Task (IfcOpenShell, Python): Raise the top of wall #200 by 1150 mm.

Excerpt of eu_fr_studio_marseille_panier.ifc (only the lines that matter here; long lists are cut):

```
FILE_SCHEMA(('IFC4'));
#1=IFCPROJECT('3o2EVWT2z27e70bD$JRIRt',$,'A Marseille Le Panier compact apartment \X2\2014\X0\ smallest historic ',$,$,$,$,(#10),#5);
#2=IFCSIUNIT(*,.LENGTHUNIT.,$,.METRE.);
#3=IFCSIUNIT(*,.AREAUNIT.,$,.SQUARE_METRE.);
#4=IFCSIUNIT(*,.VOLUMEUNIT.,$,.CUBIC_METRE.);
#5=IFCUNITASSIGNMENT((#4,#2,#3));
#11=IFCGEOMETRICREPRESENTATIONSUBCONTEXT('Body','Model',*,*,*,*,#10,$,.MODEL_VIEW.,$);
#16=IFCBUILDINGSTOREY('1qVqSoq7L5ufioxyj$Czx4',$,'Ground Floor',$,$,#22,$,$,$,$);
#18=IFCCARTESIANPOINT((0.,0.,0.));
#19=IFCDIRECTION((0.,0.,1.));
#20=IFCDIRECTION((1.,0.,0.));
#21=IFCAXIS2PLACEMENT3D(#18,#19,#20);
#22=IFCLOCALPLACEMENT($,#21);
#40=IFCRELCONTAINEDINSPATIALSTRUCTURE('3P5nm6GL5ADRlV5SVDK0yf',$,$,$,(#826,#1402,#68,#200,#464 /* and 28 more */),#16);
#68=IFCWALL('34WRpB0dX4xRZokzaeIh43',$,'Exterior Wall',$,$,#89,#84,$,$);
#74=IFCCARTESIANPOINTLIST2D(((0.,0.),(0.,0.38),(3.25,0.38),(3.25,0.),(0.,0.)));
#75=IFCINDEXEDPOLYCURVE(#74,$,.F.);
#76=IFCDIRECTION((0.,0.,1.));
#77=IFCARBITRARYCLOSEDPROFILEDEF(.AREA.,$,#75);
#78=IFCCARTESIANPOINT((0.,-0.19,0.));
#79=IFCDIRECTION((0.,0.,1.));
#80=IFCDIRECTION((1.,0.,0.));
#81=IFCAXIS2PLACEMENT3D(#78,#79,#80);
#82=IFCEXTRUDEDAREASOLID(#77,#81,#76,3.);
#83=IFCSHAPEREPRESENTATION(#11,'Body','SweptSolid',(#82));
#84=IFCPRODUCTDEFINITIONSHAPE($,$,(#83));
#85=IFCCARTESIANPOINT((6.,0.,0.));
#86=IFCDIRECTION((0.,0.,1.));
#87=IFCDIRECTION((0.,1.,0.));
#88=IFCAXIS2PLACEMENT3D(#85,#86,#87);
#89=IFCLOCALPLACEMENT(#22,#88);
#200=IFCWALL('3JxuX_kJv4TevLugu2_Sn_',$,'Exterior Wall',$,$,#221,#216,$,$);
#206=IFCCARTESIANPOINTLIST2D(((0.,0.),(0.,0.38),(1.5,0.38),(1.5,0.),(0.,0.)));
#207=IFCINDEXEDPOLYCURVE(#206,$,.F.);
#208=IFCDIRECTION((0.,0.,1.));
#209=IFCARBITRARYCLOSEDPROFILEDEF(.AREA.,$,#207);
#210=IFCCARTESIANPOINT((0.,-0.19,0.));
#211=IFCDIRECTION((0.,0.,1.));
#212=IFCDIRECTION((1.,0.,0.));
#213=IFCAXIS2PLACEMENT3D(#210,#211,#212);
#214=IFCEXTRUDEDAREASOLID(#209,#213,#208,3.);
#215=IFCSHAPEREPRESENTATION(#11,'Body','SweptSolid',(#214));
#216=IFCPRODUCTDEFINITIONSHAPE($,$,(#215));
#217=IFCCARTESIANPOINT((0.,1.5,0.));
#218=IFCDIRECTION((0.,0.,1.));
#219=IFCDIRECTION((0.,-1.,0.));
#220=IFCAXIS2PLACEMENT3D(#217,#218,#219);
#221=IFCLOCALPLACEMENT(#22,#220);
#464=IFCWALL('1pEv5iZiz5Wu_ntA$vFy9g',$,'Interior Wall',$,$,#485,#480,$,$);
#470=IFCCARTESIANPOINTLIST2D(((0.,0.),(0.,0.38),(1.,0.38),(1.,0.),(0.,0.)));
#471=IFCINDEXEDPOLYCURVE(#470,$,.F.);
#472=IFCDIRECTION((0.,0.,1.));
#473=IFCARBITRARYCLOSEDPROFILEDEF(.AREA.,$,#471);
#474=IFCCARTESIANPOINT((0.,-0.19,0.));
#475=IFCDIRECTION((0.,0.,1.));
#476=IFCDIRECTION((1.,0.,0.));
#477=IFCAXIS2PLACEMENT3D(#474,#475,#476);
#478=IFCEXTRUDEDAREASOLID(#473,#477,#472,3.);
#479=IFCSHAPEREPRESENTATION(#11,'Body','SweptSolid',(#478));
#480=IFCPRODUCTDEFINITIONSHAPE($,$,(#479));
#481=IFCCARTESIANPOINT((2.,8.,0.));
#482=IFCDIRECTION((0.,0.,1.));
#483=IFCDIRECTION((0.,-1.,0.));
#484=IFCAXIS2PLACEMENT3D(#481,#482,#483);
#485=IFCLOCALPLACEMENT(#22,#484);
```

```python
import ifcopenshell
import ifcopenshell.geom
import ifcopenshell.util.representation
import ifcopenshell.util.shape

model = ifcopenshell.open("eu_fr_studio_marseille_panier.ifc")
settings = ifcopenshell.geom.settings()


def volume(element):
    """Net volume in cubic metres, openings subtracted."""
    shape = ifcopenshell.geom.create_shape(settings, element)
    return ifcopenshell.util.shape.get_volume(shape.geometry)


wall = model.by_guid("3JxuX_kJv4TevLugu2_Sn_")
before = volume(wall)

body = ifcopenshell.util.representation.get_representation(wall, "Model", "Body")
solid = body.Items[0]
old_height = solid.Depth
solid.Depth += 1.15
after = volume(wall)

print(f"height {old_height:g} -> {solid.Depth:g}, volume {before:.3f} -> {after:.3f} m3")

model.write("eu_fr_studio_marseille_panier-out.ifc")
```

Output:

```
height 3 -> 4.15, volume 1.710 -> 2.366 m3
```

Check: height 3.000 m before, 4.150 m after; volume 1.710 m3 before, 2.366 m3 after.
